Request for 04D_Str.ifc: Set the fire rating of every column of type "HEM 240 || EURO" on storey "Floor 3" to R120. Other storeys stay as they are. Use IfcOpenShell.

First a look at what the model holds.

```python
import ifcopenshell
import ifcopenshell.util.element

model = ifcopenshell.open("04D_Str.ifc")
print(model.schema)
storey = next(s for s in model.by_type("IfcBuildingStorey") if s.Name == "Floor 3")
columns = [e for e in ifcopenshell.util.element.get_decomposition(storey) if e.is_a("IfcColumn")]
seen = {}
for e in columns:
    element_type = ifcopenshell.util.element.get_type(e)
    key = (element_type.Name if element_type != e and element_type else None, ifcopenshell.util.element.get_pset(e, "Pset_ColumnCommon", "FireRating"))
    seen[key] = seen.get(key, 0) + 1
for (name, value), count in sorted(seen.items(), key=str):
    print(count, "x", name, "|", value)
```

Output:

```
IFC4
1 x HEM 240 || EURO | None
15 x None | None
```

```python
import ifcopenshell
import ifcopenshell.api.pset
import ifcopenshell.util.element

model = ifcopenshell.open("04D_Str.ifc")

storey = next(s for s in model.by_type("IfcBuildingStorey") if s.Name == "Floor 3")
columns = [e for e in ifcopenshell.util.element.get_decomposition(storey) if e.is_a("IfcColumn")]

count = 0
for e in columns:
    element_type = ifcopenshell.util.element.get_type(e)
    if element_type in (None, e) or element_type.Name != "HEM 240 || EURO":
        continue
    # add_pset returns the element's existing set when there is one.
    pset = ifcopenshell.api.pset.add_pset(model, product=e, name="Pset_ColumnCommon")
    ifcopenshell.api.pset.edit_pset(model, pset=pset, properties={"FireRating": "R120"})
    count += 1

print(count, "columns updated")

model.write("04D_Str_v2.ifc")
```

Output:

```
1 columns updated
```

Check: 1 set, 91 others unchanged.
